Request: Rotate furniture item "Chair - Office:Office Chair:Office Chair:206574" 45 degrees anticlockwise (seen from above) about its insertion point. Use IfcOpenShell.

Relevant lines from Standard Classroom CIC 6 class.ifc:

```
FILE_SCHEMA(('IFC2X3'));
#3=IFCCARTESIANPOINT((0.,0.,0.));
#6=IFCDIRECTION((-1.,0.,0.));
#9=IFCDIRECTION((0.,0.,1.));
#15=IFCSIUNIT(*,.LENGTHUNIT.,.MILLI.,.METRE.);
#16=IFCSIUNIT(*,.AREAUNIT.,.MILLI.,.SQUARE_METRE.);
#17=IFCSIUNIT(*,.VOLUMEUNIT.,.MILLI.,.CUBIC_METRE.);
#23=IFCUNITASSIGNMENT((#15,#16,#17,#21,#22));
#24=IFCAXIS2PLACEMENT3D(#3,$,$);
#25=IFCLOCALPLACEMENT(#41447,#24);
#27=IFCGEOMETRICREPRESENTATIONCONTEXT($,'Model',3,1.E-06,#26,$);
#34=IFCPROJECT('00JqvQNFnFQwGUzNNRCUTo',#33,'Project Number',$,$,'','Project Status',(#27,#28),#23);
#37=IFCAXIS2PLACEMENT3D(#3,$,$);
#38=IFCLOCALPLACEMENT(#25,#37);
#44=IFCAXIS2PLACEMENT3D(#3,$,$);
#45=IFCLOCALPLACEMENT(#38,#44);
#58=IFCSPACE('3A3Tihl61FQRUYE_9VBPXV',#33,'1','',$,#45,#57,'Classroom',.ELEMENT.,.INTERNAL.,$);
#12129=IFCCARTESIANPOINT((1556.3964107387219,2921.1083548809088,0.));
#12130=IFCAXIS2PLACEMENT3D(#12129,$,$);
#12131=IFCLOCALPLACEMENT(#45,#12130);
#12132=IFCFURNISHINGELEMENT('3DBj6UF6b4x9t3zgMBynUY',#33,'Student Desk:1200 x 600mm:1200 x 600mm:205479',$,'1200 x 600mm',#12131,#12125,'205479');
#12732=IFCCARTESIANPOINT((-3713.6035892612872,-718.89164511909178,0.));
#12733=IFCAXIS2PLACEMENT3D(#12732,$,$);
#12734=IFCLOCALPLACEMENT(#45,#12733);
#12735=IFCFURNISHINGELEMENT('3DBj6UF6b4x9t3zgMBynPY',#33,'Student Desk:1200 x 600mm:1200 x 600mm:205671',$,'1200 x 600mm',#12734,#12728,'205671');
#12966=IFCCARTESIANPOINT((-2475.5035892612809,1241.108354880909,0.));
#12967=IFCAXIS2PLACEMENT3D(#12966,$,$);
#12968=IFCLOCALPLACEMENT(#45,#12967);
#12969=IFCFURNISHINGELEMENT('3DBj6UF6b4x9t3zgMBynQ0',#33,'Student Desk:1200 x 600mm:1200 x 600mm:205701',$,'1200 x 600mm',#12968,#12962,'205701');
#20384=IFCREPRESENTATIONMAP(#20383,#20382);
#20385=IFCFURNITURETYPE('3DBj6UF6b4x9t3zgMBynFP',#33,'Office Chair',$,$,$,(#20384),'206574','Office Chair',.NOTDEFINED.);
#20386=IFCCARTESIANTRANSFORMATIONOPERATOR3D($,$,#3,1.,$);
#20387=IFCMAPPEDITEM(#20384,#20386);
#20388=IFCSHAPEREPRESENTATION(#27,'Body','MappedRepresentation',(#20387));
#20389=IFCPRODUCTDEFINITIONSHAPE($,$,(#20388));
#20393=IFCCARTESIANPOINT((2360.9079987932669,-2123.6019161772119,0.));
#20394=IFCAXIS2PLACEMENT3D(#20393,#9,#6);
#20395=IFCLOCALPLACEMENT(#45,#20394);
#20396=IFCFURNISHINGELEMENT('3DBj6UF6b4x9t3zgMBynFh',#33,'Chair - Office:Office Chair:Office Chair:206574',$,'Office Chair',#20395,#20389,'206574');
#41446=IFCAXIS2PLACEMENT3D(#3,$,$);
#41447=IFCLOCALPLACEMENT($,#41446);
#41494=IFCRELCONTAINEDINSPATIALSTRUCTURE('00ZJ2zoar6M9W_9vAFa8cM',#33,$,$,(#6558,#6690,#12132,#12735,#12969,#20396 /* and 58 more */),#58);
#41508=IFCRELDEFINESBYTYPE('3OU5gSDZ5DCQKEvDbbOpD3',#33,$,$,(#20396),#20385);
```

```python
import ifcopenshell
import ifcopenshell.api.geometry
import ifcopenshell.util.placement

model = ifcopenshell.open("Standard Classroom CIC 6 class.ifc")

item = model.by_guid("3DBj6UF6b4x9t3zgMBynFh")
matrix = ifcopenshell.util.placement.get_local_placement(item.ObjectPlacement)
matrix = matrix @ ifcopenshell.util.placement.rotation(45, "Z")
ifcopenshell.api.geometry.edit_object_placement(model, product=item, matrix=matrix, is_si=False)

print(ifcopenshell.util.placement.get_local_placement(item.ObjectPlacement).round(3) + 0.0)

model.write("Standard Classroom CIC 6 class_v2.ifc")
```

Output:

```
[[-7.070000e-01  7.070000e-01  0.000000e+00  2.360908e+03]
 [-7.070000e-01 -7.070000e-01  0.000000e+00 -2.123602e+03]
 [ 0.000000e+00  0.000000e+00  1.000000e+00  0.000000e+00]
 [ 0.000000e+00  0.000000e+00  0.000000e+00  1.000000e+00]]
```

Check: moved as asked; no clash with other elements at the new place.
